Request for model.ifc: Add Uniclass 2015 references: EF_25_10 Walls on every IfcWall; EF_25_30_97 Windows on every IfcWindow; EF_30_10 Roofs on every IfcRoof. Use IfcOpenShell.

First a look at what the model holds.

```python
import ifcopenshell

model = ifcopenshell.open("model.ifc")
print(model.schema)
print("classifications:", [c.Name for c in model.by_type("IfcClassification")])
for ifc_class in ("IfcDoor", "IfcRoof", "IfcStair", "IfcWall", "IfcWindow"):
    print(ifc_class, len(model.by_type(ifc_class)))
```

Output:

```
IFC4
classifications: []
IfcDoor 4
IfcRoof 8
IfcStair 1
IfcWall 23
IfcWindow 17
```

```python
import ifcopenshell
import ifcopenshell.api.classification

model = ifcopenshell.open("model.ifc")

system = ifcopenshell.api.classification.add_classification(model, classification="Uniclass 2015")

codes = {
    "IfcWall": ("EF_25_10", "Walls"),
    "IfcWindow": ("EF_25_30_97", "Windows"),
    "IfcRoof": ("EF_30_10", "Roofs"),
}
for ifc_class, (code, name) in codes.items():
    products = model.by_type(ifc_class)
    ifcopenshell.api.classification.add_reference(
        model, products=products, classification=system, identification=code, name=name
    )
    print(code, len(products))

model.write("model_updated.ifc")
```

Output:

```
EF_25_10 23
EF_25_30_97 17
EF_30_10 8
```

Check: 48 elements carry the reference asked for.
